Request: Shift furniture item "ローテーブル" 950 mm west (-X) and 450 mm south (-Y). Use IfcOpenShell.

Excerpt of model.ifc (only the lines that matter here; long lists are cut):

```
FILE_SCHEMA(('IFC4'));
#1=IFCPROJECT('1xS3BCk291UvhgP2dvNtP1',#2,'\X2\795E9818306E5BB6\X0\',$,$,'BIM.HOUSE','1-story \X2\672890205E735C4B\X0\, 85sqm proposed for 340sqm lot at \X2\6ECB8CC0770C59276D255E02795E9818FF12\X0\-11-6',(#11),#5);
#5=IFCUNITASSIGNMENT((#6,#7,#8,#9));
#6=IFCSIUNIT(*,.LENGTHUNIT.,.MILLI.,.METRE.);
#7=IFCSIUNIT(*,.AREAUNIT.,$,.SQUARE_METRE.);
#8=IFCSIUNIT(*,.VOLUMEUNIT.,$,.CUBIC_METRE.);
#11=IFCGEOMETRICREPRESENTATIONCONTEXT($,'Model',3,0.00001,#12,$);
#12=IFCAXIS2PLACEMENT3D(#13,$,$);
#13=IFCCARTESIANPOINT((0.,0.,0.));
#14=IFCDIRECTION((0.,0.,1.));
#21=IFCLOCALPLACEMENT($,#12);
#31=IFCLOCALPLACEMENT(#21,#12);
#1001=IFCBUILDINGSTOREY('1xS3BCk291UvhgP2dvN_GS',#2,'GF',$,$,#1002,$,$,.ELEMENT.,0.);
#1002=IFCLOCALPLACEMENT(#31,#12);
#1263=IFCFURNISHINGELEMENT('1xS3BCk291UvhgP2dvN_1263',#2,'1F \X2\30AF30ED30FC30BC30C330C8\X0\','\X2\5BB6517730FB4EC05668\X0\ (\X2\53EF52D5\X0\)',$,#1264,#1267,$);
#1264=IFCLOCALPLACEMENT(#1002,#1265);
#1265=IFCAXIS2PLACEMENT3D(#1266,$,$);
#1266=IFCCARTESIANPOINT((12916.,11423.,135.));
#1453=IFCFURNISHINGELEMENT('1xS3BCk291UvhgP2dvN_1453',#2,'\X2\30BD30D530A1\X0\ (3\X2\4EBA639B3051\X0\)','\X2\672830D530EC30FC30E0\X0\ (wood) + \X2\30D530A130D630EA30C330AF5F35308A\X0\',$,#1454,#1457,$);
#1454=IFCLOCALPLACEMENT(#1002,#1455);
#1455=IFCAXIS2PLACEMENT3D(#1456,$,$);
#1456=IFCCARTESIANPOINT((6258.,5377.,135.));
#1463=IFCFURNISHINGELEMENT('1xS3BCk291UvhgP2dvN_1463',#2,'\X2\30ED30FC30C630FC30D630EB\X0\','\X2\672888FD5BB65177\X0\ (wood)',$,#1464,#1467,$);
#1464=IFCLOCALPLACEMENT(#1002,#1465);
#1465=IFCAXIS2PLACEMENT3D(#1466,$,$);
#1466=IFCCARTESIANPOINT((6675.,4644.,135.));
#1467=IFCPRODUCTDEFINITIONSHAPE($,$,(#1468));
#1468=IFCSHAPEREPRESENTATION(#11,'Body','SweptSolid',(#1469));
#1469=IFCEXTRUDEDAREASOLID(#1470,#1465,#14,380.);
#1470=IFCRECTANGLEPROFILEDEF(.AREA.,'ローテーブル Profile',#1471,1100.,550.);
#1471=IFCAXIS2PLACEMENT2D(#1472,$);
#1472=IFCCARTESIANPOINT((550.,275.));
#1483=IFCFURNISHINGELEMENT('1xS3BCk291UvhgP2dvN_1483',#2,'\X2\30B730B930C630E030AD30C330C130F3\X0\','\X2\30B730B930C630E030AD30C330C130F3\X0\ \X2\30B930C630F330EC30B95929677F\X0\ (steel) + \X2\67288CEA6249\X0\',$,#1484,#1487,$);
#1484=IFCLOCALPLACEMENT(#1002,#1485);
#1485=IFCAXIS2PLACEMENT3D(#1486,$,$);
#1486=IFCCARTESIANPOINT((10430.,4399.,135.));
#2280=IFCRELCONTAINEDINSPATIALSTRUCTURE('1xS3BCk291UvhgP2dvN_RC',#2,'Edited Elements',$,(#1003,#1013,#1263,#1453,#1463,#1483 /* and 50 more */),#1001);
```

```python
import ifcopenshell
import ifcopenshell.api.geometry
import ifcopenshell.util.placement
import ifcopenshell.util.unit

model = ifcopenshell.open("model.ifc")
unit_scale = ifcopenshell.util.unit.calculate_unit_scale(model)

item = model.by_id(1463)
matrix = ifcopenshell.util.placement.get_local_placement(item.ObjectPlacement)
matrix[0, 3] -= 0.95 / unit_scale
matrix[1, 3] -= 0.45 / unit_scale
ifcopenshell.api.geometry.edit_object_placement(model, product=item, matrix=matrix, is_si=False)

print(ifcopenshell.util.placement.get_local_placement(item.ObjectPlacement).round(3) + 0.0)

model.write("model_edited.ifc")
```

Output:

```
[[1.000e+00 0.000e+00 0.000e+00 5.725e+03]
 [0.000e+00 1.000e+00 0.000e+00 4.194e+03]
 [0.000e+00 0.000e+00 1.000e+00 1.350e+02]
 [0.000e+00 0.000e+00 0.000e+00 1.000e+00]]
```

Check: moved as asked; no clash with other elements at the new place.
